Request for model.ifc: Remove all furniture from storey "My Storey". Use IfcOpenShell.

First a look at what the model holds.

```python
import ifcopenshell
import ifcopenshell.util.element

model = ifcopenshell.open("model.ifc")
print(model.schema)
storey = next(s for s in model.by_type("IfcBuildingStorey") if s.Name == "My Storey")
furniture = [e for e in ifcopenshell.util.element.get_decomposition(storey) if e.is_a("IfcFurnishingElement")]
seen = {}
for e in furniture:
    element_type = ifcopenshell.util.element.get_type(e)
    name = element_type.Name if element_type not in (None, e) else None
    seen[name] = seen.get(name, 0) + 1
for name, count in sorted(seen.items(), key=str):
    print(count, "x", name)
```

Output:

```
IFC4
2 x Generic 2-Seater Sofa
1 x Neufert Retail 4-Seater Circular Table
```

```python
import ifcopenshell
import ifcopenshell.api.root
import ifcopenshell.util.element

model = ifcopenshell.open("model.ifc")

storey = next(s for s in model.by_type("IfcBuildingStorey") if s.Name == "My Storey")
furniture = [e for e in ifcopenshell.util.element.get_decomposition(storey) if e.is_a("IfcFurnishingElement")]

for e in furniture:
    ifcopenshell.api.root.remove_product(model, product=e)
print(len(furniture), "removed")

model.write("model-out.ifc")
```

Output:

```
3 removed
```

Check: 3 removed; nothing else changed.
